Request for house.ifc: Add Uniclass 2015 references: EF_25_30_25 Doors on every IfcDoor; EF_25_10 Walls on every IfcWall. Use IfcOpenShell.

First a look at what the model holds.

```python
import ifcopenshell

model = ifcopenshell.open("house.ifc")
print(model.schema)
print("classifications:", [c.Name for c in model.by_type("IfcClassification")])
for ifc_class in ("IfcDoor", "IfcRoof", "IfcStair", "IfcWall", "IfcWindow"):
    print(ifc_class, len(model.by_type(ifc_class)))
```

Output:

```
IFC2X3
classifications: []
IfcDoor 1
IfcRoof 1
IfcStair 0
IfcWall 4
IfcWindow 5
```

```python
import ifcopenshell
import ifcopenshell.api.classification

model = ifcopenshell.open("house.ifc")

# IFC2X3 requires Source and Edition and has no link from the project to the system.
system = model.create_entity("IfcClassification", Source="NBS", Edition="2015", Name="Uniclass 2015")

codes = {
    "IfcDoor": ("EF_25_30_25", "Doors"),
    "IfcWall": ("EF_25_10", "Walls"),
}
for ifc_class, (code, name) in codes.items():
    products = model.by_type(ifc_class)
    ifcopenshell.api.classification.add_reference(
        model, products=products, classification=system, identification=code, name=name
    )
    print(code, len(products))

model.write("house_updated.ifc")
```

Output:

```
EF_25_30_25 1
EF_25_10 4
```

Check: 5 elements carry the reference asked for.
